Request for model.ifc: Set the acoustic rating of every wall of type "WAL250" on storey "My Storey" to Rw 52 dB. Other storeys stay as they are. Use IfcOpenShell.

First a look at what the model holds.

```python
import ifcopenshell
import ifcopenshell.util.element

model = ifcopenshell.open("model.ifc")
print(model.schema)
storey = next(s for s in model.by_type("IfcBuildingStorey") if s.Name == "My Storey")
walls = [e for e in ifcopenshell.util.element.get_decomposition(storey) if e.is_a("IfcWall")]
seen = {}
for e in walls:
    element_type = ifcopenshell.util.element.get_type(e)
    key = (element_type.Name if element_type != e and element_type else None, ifcopenshell.util.element.get_pset(e, "Pset_WallCommon", "AcousticRating"))
    seen[key] = seen.get(key, 0) + 1
for (name, value), count in sorted(seen.items(), key=str):
    print(count, "x", name, "|", value)
```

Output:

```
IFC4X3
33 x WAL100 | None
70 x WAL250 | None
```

```python
import ifcopenshell
import ifcopenshell.api.pset
import ifcopenshell.util.element

model = ifcopenshell.open("model.ifc")

storey = next(s for s in model.by_type("IfcBuildingStorey") if s.Name == "My Storey")
walls = [e for e in ifcopenshell.util.element.get_decomposition(storey) if e.is_a("IfcWall")]

count = 0
for e in walls:
    element_type = ifcopenshell.util.element.get_type(e)
    if element_type in (None, e) or element_type.Name != "WAL250":
        continue
    # add_pset returns the element's existing set when there is one.
    pset = ifcopenshell.api.pset.add_pset(model, product=e, name="Pset_WallCommon")
    ifcopenshell.api.pset.edit_pset(model, pset=pset, properties={"AcousticRating": "Rw 52 dB"})
    count += 1

print(count, "walls updated")

model.write("model-out.ifc")
```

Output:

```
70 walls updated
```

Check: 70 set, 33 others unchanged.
